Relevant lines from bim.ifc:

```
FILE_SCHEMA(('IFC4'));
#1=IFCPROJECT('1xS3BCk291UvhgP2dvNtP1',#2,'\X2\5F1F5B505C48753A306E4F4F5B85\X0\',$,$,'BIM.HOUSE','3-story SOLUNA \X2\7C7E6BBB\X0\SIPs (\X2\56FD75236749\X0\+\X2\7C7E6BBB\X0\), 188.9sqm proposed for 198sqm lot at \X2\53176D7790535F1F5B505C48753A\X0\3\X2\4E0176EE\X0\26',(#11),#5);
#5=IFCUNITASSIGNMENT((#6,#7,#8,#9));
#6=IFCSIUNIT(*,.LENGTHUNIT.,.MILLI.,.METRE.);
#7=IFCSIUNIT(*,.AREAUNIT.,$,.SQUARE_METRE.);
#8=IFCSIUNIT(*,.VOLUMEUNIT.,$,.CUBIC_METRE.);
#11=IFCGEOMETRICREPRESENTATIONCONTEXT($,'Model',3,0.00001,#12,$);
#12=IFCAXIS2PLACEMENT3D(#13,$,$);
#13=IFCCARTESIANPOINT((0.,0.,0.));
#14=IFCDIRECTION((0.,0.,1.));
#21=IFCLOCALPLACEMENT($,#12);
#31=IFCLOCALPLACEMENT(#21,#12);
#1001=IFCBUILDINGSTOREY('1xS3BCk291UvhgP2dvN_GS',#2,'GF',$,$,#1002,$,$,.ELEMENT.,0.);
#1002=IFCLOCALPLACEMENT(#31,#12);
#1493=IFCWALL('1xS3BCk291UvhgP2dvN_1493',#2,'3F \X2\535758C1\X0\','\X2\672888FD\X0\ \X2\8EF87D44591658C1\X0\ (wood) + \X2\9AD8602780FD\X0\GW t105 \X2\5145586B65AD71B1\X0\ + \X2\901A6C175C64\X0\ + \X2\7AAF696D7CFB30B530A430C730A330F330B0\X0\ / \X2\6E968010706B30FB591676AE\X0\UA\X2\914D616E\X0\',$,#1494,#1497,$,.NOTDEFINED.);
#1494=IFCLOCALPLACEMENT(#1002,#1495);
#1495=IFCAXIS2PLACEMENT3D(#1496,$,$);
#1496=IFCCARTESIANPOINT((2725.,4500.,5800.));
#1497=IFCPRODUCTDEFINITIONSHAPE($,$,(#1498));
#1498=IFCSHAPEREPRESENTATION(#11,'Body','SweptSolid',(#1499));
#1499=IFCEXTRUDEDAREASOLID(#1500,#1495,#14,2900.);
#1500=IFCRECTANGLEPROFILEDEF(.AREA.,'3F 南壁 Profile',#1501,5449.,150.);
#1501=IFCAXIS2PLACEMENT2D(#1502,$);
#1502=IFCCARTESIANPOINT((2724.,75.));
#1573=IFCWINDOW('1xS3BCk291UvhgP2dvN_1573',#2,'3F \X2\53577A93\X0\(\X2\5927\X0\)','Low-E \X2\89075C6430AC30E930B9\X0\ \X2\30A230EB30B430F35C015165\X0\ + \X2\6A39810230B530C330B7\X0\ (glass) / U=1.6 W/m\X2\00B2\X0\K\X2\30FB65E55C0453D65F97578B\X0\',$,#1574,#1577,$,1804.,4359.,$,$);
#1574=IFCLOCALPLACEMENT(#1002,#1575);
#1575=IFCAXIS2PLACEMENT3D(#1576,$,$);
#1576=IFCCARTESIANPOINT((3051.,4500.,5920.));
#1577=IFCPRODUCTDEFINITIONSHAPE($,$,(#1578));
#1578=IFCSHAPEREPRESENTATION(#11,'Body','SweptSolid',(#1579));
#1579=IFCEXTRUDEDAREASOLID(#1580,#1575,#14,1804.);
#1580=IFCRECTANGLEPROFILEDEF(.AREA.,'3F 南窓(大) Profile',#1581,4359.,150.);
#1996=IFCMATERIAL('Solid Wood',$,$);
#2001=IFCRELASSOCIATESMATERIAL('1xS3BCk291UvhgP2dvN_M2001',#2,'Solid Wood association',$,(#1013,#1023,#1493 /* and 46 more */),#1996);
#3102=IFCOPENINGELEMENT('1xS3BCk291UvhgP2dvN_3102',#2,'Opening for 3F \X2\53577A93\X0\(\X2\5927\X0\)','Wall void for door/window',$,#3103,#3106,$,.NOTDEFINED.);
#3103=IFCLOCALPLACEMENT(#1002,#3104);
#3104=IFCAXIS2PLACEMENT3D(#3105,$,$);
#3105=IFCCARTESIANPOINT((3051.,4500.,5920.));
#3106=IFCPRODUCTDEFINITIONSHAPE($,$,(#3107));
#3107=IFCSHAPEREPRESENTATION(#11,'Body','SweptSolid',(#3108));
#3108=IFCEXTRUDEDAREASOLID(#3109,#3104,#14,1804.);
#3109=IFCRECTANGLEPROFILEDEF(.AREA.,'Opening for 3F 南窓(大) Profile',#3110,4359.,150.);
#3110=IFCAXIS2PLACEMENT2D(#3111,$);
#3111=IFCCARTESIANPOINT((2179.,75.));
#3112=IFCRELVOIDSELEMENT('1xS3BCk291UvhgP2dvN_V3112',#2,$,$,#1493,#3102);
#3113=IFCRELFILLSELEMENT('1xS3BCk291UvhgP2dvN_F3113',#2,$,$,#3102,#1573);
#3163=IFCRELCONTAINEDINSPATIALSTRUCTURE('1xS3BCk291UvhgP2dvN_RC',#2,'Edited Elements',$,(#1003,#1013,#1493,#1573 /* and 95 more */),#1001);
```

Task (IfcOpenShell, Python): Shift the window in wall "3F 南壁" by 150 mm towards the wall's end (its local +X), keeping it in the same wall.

```python
import ifcopenshell
import ifcopenshell.api.geometry
import ifcopenshell.util.placement
import ifcopenshell.util.unit

model = ifcopenshell.open("bim.ifc")
unit_scale = ifcopenshell.util.unit.calculate_unit_scale(model)

window = model.by_guid("1xS3BCk291UvhgP2dvN_1573")
opening = window.FillsVoids[0].RelatingOpeningElement
wall = opening.VoidsElements[0].RelatingBuildingElement

wall_matrix = ifcopenshell.util.placement.get_local_placement(wall.ObjectPlacement)
shift = wall_matrix[:3, 0] * 0.15 / unit_scale
before = ifcopenshell.util.placement.get_local_placement(window.ObjectPlacement)[:3, 3].copy()

# The window is not placed relative to its opening, so move both.
for product in (opening, window):
    matrix = ifcopenshell.util.placement.get_local_placement(product.ObjectPlacement)
    matrix[:3, 3] += shift
    ifcopenshell.api.geometry.edit_object_placement(model, product=product, matrix=matrix, is_si=False)

after = ifcopenshell.util.placement.get_local_placement(window.ObjectPlacement)[:3, 3]
print("window moved by", (after - before).round(3) + 0.0)

model.write("bim-out.ifc")
```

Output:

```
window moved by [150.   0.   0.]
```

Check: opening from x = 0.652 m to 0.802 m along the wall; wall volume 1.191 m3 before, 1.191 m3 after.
